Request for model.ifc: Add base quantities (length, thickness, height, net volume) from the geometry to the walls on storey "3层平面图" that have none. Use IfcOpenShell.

First a look at what the model holds.

```python
import ifcopenshell
import ifcopenshell.util.element
import ifcopenshell.util.unit

model = ifcopenshell.open("model.ifc")
print(model.schema)
for unit_type in ("LENGTHUNIT", "AREAUNIT", "VOLUMEUNIT"):
    print(unit_type, ifcopenshell.util.unit.calculate_unit_scale(model, unit_type))
storey = next(s for s in model.by_type("IfcBuildingStorey") if s.Name == "3层平面图")
walls = [e for e in ifcopenshell.util.element.get_decomposition(storey) if e.is_a("IfcWall")]
for e in sorted(walls, key=lambda e: e.id()):
    print(e.id(), e.is_a(), e.Name, list(ifcopenshell.util.element.get_psets(e, qtos_only=True)), sep=" | ")
```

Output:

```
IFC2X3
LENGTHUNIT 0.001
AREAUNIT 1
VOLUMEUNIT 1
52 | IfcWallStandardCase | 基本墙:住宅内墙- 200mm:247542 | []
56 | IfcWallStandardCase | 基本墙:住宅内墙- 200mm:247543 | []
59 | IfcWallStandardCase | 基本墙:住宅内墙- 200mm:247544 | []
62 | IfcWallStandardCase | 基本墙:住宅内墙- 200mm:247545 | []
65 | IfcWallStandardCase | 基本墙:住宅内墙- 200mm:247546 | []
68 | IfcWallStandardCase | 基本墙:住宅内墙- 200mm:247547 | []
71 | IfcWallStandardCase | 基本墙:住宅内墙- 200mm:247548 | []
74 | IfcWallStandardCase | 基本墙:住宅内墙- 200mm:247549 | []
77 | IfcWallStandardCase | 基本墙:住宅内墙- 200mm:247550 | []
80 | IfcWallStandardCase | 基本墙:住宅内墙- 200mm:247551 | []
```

```python
import ifcopenshell
import ifcopenshell.api.pset
import ifcopenshell.geom
import ifcopenshell.util.element
import ifcopenshell.util.shape
import ifcopenshell.util.unit

model = ifcopenshell.open("model.ifc")
unit_scale = ifcopenshell.util.unit.calculate_unit_scale(model)
volume_scale = ifcopenshell.util.unit.calculate_unit_scale(model, "VOLUMEUNIT")
settings = ifcopenshell.geom.settings()

storey = next(s for s in model.by_type("IfcBuildingStorey") if s.Name == "3层平面图")
walls = [e for e in ifcopenshell.util.element.get_decomposition(storey) if e.is_a("IfcWall")]

for e in sorted(walls, key=lambda e: e.id()):
    if ifcopenshell.util.element.get_psets(e, qtos_only=True, should_inherit=False):
        continue
    # Geometry comes back in metres, in the element's own axes.
    shape = ifcopenshell.geom.create_shape(settings, e)
    values = {
        "Length": ifcopenshell.util.shape.get_x(shape.geometry) / unit_scale,
        "Width": ifcopenshell.util.shape.get_y(shape.geometry) / unit_scale,
        "Height": ifcopenshell.util.shape.get_z(shape.geometry) / unit_scale,
        "NetVolume": ifcopenshell.util.shape.get_volume(shape.geometry) / volume_scale,
    }
    qto = ifcopenshell.api.pset.add_qto(model, product=e, name="BaseQuantities")
    ifcopenshell.api.pset.edit_qto(model, qto=qto, properties=values)
    print(e.id(), {k: round(v, 3) for k, v in values.items()})

model.write("model_edited.ifc")
```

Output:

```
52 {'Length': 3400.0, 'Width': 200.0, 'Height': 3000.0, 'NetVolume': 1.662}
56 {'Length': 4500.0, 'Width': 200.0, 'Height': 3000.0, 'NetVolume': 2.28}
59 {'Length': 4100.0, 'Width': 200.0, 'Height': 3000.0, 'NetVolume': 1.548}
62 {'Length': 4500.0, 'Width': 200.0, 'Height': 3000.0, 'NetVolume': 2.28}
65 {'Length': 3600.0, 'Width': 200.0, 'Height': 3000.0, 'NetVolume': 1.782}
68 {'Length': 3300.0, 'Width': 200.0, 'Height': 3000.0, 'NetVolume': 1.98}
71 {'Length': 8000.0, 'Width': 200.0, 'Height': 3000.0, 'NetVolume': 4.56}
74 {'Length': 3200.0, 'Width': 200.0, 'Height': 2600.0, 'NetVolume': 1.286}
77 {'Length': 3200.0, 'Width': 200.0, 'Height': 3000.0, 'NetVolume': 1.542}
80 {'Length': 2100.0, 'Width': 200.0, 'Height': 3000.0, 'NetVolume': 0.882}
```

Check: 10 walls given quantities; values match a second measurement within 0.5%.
